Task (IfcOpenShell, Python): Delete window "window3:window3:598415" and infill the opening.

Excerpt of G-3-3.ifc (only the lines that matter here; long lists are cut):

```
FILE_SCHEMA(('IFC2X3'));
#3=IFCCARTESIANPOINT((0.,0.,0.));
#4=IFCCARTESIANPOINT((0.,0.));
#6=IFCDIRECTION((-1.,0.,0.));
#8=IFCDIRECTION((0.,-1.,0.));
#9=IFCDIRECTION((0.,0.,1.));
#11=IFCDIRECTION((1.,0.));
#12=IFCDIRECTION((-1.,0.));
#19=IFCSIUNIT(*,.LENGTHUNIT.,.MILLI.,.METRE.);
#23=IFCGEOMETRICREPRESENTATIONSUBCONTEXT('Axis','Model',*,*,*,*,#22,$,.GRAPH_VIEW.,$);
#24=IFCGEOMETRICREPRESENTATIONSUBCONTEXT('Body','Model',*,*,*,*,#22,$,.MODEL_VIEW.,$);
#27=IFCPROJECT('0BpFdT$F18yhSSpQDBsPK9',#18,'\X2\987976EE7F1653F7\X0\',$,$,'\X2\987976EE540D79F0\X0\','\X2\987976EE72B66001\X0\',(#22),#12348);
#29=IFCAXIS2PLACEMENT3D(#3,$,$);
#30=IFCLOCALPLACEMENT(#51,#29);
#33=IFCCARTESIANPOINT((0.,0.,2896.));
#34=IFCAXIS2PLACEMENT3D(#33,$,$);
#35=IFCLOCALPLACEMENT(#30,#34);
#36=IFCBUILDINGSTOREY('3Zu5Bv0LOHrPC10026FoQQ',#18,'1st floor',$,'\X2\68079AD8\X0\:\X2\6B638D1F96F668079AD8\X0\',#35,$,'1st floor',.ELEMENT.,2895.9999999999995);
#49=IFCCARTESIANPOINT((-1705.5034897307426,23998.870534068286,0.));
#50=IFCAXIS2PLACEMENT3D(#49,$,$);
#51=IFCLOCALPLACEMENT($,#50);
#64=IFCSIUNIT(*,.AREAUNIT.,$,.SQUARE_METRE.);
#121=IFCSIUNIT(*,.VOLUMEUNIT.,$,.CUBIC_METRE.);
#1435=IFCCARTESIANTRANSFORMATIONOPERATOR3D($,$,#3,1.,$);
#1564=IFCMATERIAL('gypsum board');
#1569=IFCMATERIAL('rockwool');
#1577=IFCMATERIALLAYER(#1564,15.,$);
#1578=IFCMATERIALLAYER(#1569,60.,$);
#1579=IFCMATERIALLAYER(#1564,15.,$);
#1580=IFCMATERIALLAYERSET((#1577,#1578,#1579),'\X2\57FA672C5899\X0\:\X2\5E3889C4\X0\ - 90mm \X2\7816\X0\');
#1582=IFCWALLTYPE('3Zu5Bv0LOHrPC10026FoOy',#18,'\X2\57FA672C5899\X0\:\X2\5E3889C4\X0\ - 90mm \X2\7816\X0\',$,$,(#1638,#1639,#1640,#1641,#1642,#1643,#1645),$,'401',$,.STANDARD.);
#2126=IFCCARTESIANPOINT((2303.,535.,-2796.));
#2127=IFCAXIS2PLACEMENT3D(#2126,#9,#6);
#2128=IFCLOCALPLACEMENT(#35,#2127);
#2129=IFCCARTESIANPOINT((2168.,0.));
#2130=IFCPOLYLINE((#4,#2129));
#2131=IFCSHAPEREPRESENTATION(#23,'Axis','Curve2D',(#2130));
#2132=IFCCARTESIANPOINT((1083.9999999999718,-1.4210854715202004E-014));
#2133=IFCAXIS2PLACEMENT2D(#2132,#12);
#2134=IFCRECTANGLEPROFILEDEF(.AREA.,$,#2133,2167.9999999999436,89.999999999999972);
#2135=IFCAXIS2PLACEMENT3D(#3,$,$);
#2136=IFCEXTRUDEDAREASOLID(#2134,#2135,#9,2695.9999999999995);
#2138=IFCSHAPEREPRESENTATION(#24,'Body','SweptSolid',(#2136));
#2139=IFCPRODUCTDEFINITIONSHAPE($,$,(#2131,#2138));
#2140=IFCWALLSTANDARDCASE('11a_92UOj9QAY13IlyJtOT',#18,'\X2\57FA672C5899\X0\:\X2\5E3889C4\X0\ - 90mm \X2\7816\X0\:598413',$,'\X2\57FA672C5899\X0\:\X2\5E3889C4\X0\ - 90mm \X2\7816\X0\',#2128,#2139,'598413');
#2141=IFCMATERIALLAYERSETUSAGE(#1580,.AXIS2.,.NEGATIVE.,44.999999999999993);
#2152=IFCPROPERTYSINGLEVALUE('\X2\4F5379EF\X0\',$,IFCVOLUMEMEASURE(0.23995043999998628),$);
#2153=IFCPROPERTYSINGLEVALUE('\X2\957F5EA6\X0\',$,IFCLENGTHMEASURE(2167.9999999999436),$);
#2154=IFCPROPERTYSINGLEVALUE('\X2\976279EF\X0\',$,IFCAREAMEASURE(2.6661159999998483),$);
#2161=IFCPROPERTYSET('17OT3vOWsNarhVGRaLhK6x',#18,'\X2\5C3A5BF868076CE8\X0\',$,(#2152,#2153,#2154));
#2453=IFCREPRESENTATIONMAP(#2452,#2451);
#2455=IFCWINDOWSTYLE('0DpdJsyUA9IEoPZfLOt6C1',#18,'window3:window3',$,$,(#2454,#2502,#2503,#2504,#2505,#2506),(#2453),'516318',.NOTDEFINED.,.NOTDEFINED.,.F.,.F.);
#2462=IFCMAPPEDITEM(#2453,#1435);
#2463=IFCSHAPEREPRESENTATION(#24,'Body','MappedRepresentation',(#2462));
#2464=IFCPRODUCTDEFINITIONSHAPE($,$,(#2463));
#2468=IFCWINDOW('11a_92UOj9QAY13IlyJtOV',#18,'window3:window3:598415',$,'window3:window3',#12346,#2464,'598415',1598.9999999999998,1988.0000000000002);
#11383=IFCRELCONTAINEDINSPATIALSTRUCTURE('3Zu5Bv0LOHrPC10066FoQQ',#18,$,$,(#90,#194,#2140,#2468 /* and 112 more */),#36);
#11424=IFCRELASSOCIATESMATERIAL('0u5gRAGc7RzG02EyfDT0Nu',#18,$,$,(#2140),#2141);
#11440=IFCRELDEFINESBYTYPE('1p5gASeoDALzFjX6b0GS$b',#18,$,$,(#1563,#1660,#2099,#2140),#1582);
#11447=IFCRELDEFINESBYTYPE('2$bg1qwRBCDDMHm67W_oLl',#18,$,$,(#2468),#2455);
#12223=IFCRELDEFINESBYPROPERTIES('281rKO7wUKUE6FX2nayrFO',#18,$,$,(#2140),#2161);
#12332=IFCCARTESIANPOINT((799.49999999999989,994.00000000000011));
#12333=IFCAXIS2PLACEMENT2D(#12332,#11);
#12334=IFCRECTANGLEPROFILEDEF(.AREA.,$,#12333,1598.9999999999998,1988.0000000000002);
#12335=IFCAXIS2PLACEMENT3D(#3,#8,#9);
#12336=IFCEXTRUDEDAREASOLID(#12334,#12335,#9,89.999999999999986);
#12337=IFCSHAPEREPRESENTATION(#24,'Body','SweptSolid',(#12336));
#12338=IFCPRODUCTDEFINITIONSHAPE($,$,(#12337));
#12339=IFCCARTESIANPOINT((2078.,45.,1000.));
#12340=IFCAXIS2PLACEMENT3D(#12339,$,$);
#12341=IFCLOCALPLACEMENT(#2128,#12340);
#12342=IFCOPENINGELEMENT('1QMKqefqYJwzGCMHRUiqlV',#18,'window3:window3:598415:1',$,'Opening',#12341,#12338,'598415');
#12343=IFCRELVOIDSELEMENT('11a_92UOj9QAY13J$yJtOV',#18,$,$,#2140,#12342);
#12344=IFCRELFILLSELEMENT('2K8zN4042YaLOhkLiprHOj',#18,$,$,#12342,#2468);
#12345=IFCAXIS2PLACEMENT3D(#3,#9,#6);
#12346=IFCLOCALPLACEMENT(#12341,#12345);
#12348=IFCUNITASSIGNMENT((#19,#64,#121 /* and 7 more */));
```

```python
import ifcopenshell
import ifcopenshell.api.feature
import ifcopenshell.api.pset
import ifcopenshell.api.root
import ifcopenshell.geom
import ifcopenshell.util.element
import ifcopenshell.util.shape
import ifcopenshell.util.unit

model = ifcopenshell.open("G-3-3.ifc")
area_scale = ifcopenshell.util.unit.calculate_unit_scale(model, "AREAUNIT")
volume_scale = ifcopenshell.util.unit.calculate_unit_scale(model, "VOLUMEUNIT")
settings = ifcopenshell.geom.settings()


def volume(element):
    """Net volume in cubic metres, openings subtracted."""
    shape = ifcopenshell.geom.create_shape(settings, element)
    return ifcopenshell.util.shape.get_volume(shape.geometry)


window = model.by_guid("11a_92UOj9QAY13IlyJtOV")
opening = window.FillsVoids[0].RelatingOpeningElement
wall = opening.VoidsElements[0].RelatingBuildingElement
before = volume(wall)

ifcopenshell.api.root.remove_product(model, product=window)
ifcopenshell.api.feature.remove_feature(model, feature=opening)

after = volume(wall)
thickness = 0.09  # wall thickness in metres

# Update the wall's stored quantities.
pset = model.by_id(ifcopenshell.util.element.get_pset(wall, "尺寸标注", should_inherit=False)["id"])
ifcopenshell.api.pset.edit_pset(model, pset=pset, properties={
    "体积": model.create_entity("IfcVolumeMeasure", after / volume_scale),
    "面积": model.create_entity("IfcAreaMeasure", after / thickness / area_scale),
})

print(f"wall volume {before:.3f} -> {after:.3f} m3")

model.write("G-3-3_edited.ifc")
```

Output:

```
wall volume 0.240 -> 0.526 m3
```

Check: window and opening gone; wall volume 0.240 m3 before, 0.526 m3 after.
